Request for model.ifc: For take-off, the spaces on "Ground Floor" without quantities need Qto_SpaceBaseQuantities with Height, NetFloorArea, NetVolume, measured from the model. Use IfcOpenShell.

First a look at what the model holds.

```python
import ifcopenshell
import ifcopenshell.util.element
import ifcopenshell.util.unit

model = ifcopenshell.open("model.ifc")
print(model.schema)
for unit_type in ("LENGTHUNIT", "AREAUNIT", "VOLUMEUNIT"):
    print(unit_type, ifcopenshell.util.unit.calculate_unit_scale(model, unit_type))
storey = next(s for s in model.by_type("IfcBuildingStorey") if s.Name == "Ground Floor")
spaces = [e for e in ifcopenshell.util.element.get_decomposition(storey) if e.is_a("IfcSpace")]
for e in sorted(spaces, key=lambda e: e.id()):
    print(e.id(), e.is_a(), e.Name, list(ifcopenshell.util.element.get_psets(e, qtos_only=True)), sep=" | ")
```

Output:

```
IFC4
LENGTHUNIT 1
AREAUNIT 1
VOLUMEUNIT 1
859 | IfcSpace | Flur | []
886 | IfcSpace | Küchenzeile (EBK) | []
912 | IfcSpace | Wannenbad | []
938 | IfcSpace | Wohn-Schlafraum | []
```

```python
import ifcopenshell
import ifcopenshell.api.pset
import ifcopenshell.geom
import ifcopenshell.util.element
import ifcopenshell.util.shape
import ifcopenshell.util.unit

model = ifcopenshell.open("model.ifc")
unit_scale = ifcopenshell.util.unit.calculate_unit_scale(model)
area_scale = ifcopenshell.util.unit.calculate_unit_scale(model, "AREAUNIT")
volume_scale = ifcopenshell.util.unit.calculate_unit_scale(model, "VOLUMEUNIT")
settings = ifcopenshell.geom.settings()

storey = next(s for s in model.by_type("IfcBuildingStorey") if s.Name == "Ground Floor")
spaces = [e for e in ifcopenshell.util.element.get_decomposition(storey) if e.is_a("IfcSpace")]

for e in sorted(spaces, key=lambda e: e.id()):
    if ifcopenshell.util.element.get_psets(e, qtos_only=True, should_inherit=False):
        continue
    # Geometry comes back in metres, in the element's own axes.
    shape = ifcopenshell.geom.create_shape(settings, e)
    values = {
        "Height": ifcopenshell.util.shape.get_z(shape.geometry) / unit_scale,
        "NetFloorArea": ifcopenshell.util.shape.get_footprint_area(shape.geometry) / area_scale,
        "NetVolume": ifcopenshell.util.shape.get_volume(shape.geometry) / volume_scale,
    }
    qto = ifcopenshell.api.pset.add_qto(model, product=e, name="Qto_SpaceBaseQuantities")
    ifcopenshell.api.pset.edit_qto(model, qto=qto, properties=values)
    print(e.id(), {k: round(v, 3) for k, v in values.items()})

model.write("model_updated.ifc")
```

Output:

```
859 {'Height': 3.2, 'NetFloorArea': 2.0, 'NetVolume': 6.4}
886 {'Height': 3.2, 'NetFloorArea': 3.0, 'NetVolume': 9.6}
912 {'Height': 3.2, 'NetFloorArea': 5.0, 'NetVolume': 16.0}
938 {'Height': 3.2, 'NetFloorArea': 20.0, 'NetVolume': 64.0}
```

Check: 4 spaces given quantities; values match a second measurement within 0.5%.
